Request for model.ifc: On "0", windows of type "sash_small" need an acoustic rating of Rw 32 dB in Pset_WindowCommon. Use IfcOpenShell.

First a look at what the model holds.

```python
import ifcopenshell
import ifcopenshell.util.element

model = ifcopenshell.open("model.ifc")
print(model.schema)
storey = next(s for s in model.by_type("IfcBuildingStorey") if s.Name == "0")
windows = [e for e in ifcopenshell.util.element.get_decomposition(storey) if e.is_a("IfcWindow")]
seen = {}
for e in windows:
    element_type = ifcopenshell.util.element.get_type(e)
    key = (element_type.Name if element_type != e and element_type else None, ifcopenshell.util.element.get_pset(e, "Pset_WindowCommon", "AcousticRating"))
    seen[key] = seen.get(key, 0) + 1
for (name, value), count in sorted(seen.items(), key=str):
    print(count, "x", name, "|", value)
```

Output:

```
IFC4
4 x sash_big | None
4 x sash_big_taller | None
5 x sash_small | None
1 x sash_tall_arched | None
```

```python
import ifcopenshell
import ifcopenshell.api.pset
import ifcopenshell.util.element

model = ifcopenshell.open("model.ifc")

storey = next(s for s in model.by_type("IfcBuildingStorey") if s.Name == "0")
windows = [e for e in ifcopenshell.util.element.get_decomposition(storey) if e.is_a("IfcWindow")]

count = 0
for e in windows:
    element_type = ifcopenshell.util.element.get_type(e)
    if element_type in (None, e) or element_type.Name != "sash_small":
        continue
    # add_pset returns the element's existing set when there is one.
    pset = ifcopenshell.api.pset.add_pset(model, product=e, name="Pset_WindowCommon")
    ifcopenshell.api.pset.edit_pset(model, pset=pset, properties={"AcousticRating": "Rw 32 dB"})
    count += 1

print(count, "windows updated")

model.write("model_v2.ifc")
```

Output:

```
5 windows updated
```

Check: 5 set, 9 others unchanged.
